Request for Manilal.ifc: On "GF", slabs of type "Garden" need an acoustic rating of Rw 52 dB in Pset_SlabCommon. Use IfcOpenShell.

First a look at what the model holds.

```python
import ifcopenshell
import ifcopenshell.util.element

model = ifcopenshell.open("Manilal.ifc")
print(model.schema)
storey = next(s for s in model.by_type("IfcBuildingStorey") if s.Name == "GF")
slabs = [e for e in ifcopenshell.util.element.get_decomposition(storey) if e.is_a("IfcSlab")]
seen = {}
for e in slabs:
    element_type = ifcopenshell.util.element.get_type(e)
    key = (element_type.Name if element_type != e and element_type else None, ifcopenshell.util.element.get_pset(e, "Pset_SlabCommon", "AcousticRating"))
    seen[key] = seen.get(key, 0) + 1
for (name, value), count in sorted(seen.items(), key=str):
    print(count, "x", name, "|", value)
```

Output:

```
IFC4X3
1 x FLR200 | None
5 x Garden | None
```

```python
import ifcopenshell
import ifcopenshell.api.pset
import ifcopenshell.util.element

model = ifcopenshell.open("Manilal.ifc")

storey = next(s for s in model.by_type("IfcBuildingStorey") if s.Name == "GF")
slabs = [e for e in ifcopenshell.util.element.get_decomposition(storey) if e.is_a("IfcSlab")]

count = 0
for e in slabs:
    element_type = ifcopenshell.util.element.get_type(e)
    if element_type in (None, e) or element_type.Name != "Garden":
        continue
    # add_pset returns the element's existing set when there is one.
    pset = ifcopenshell.api.pset.add_pset(model, product=e, name="Pset_SlabCommon")
    ifcopenshell.api.pset.edit_pset(model, pset=pset, properties={"AcousticRating": "Rw 52 dB"})
    count += 1

print(count, "slabs updated")

model.write("Manilal_v2.ifc")
```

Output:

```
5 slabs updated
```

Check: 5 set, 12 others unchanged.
